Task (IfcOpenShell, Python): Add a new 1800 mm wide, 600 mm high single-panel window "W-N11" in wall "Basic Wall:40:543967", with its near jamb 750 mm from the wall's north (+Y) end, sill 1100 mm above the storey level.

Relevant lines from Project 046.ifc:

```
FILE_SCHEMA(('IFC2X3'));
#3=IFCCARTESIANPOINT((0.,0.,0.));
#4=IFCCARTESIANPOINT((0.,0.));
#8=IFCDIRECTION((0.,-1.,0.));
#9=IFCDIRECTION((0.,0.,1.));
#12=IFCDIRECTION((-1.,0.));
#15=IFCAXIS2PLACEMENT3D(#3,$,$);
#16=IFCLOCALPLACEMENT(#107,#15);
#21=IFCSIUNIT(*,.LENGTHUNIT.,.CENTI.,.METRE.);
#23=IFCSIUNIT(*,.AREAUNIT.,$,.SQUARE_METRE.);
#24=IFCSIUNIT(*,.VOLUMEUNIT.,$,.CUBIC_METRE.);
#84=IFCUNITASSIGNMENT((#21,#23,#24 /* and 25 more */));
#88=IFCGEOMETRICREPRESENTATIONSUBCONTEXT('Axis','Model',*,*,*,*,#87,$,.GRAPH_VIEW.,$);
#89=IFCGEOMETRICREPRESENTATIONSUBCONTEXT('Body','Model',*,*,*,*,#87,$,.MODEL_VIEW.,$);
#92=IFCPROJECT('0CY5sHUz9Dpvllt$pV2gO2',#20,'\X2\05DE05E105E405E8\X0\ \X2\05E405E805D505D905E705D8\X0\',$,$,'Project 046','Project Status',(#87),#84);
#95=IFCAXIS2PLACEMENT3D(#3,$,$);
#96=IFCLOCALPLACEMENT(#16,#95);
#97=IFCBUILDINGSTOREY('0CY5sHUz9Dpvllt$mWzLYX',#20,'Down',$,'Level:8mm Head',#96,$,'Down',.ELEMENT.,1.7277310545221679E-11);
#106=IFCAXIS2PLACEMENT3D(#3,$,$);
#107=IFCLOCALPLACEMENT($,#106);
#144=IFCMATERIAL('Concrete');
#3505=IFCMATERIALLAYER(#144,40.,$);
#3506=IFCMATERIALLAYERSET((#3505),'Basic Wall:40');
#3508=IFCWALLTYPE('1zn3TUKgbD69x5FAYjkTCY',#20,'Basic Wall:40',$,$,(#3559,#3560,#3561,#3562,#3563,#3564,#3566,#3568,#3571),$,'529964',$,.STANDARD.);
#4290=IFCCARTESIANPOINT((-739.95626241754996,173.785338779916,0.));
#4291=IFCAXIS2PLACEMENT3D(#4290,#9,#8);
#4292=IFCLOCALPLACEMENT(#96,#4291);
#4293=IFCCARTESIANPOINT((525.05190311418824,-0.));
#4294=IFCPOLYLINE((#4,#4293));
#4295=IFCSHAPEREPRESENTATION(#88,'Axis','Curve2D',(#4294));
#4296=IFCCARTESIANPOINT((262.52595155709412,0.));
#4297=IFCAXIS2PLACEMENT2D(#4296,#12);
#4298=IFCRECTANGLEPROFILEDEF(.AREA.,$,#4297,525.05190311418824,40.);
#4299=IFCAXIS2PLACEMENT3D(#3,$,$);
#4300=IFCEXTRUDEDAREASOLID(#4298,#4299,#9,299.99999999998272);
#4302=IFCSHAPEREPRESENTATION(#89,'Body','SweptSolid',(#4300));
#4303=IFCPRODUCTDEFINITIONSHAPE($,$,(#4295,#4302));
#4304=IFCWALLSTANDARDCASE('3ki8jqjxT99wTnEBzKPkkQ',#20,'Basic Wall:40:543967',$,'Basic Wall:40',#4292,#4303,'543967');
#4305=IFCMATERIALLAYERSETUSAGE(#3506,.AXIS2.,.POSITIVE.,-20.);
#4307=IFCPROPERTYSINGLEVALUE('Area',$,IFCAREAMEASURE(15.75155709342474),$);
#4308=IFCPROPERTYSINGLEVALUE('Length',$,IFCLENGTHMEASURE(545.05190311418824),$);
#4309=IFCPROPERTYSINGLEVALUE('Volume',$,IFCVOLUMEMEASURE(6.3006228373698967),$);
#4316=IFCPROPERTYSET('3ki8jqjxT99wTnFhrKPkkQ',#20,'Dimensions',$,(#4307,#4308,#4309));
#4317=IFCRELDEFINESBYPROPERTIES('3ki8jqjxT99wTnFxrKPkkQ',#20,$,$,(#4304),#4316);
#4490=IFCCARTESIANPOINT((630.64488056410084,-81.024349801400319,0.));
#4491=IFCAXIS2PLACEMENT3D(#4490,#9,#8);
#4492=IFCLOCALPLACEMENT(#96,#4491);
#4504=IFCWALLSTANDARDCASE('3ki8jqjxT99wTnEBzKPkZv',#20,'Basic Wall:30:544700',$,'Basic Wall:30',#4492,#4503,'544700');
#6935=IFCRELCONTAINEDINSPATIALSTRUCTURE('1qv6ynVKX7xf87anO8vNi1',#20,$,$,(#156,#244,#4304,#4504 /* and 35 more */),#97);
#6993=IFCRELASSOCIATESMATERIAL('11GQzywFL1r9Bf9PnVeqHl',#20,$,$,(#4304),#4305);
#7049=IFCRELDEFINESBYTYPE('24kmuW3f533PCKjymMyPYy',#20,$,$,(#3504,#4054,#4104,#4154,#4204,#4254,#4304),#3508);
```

```python
import numpy as np
import ifcopenshell
import ifcopenshell.api.feature
import ifcopenshell.api.geometry
import ifcopenshell.api.pset
import ifcopenshell.api.root
import ifcopenshell.api.spatial
import ifcopenshell.api.type
import ifcopenshell.geom
import ifcopenshell.util.element
import ifcopenshell.util.placement
import ifcopenshell.util.representation
import ifcopenshell.util.shape
import ifcopenshell.util.unit

model = ifcopenshell.open("Project 046.ifc")
unit_scale = ifcopenshell.util.unit.calculate_unit_scale(model)
area_scale = ifcopenshell.util.unit.calculate_unit_scale(model, "AREAUNIT")
volume_scale = ifcopenshell.util.unit.calculate_unit_scale(model, "VOLUMEUNIT")
settings = ifcopenshell.geom.settings()


def volume(element):
    """Net volume in cubic metres, openings subtracted."""
    shape = ifcopenshell.geom.create_shape(settings, element)
    return ifcopenshell.util.shape.get_volume(shape.geometry)


wall = model.by_guid("3ki8jqjxT99wTnEBzKPkkQ")
storey = ifcopenshell.util.element.get_container(wall, ifc_class="IfcBuildingStorey")
context = ifcopenshell.util.representation.get_context(model, "Model", "Body", "MODEL_VIEW")
before = volume(wall)

width, height, from_end, sill = 1.8, 0.6, 0.75, 1.1  # metres

# The wall runs along its own X axis, and the end named is its -X end.
wall_shape = ifcopenshell.geom.create_shape(settings, wall)
x, y, z = ifcopenshell.util.shape.get_vertices(wall_shape.geometry).T
start = x.min() + from_end
face, thickness = float(y.min()), float(y.max() - y.min())
wall_matrix = ifcopenshell.util.placement.get_local_placement(wall.ObjectPlacement)
level = ifcopenshell.util.placement.get_local_placement(storey.ObjectPlacement)[2, 3]


def in_wall(x, y):
    """Placement at x, y metres in the wall's axes, at sill height."""
    matrix = wall_matrix.copy()
    matrix[:, 3] = wall_matrix @ np.array([x / unit_scale, y / unit_scale, 0.0, 1.0])
    matrix[2, 3] = level + sill / unit_scale
    return matrix


# Opening: a box that overshoots both wall faces by 50 mm.
opening = ifcopenshell.api.root.create_entity(model, ifc_class="IfcOpeningElement")
box = ifcopenshell.api.geometry.add_wall_representation(
    model, context=context, length=width, height=height, thickness=thickness + 0.1
)
ifcopenshell.api.geometry.assign_representation(model, product=opening, representation=box)
ifcopenshell.api.geometry.edit_object_placement(model, product=opening, matrix=in_wall(start, face - 0.05), is_si=False)
ifcopenshell.api.feature.add_feature(model, feature=opening, element=wall)

window = ifcopenshell.api.root.create_entity(model, ifc_class="IfcWindow", name="W-N11")
window.OverallWidth, window.OverallHeight = width / unit_scale, height / unit_scale
body = ifcopenshell.api.geometry.add_window_representation(
    model,
    context=context,
    overall_width=window.OverallWidth,
    overall_height=window.OverallHeight,
    partition_type="SINGLE_PANEL",
)
ifcopenshell.api.geometry.assign_representation(model, product=window, representation=body)
ifcopenshell.api.spatial.assign_container(model, products=[window], relating_structure=storey)
fills = ifcopenshell.api.feature.add_filling(model, opening=opening, element=window)
fills.OwnerHistory = window.OwnerHistory  # required in IFC2X3

# IFC2X3 keeps the operation on the window style.
style = ifcopenshell.api.root.create_entity(model, ifc_class="IfcWindowStyle", name="W-N11")
style.OperationType, style.ConstructionType = "SINGLE_PANEL", "NOTDEFINED"
style.ParameterTakesPrecedence = style.Sizeable = False
ifcopenshell.api.type.assign_type(model, related_objects=[window], relating_type=style)

# Centre the window in the wall's thickness.
ifcopenshell.api.geometry.edit_object_placement(model, product=window, matrix=in_wall(start, face), is_si=False)
window_shape = ifcopenshell.geom.create_shape(settings, window)
depth = ifcopenshell.util.shape.get_vertices(window_shape.geometry)[:, 1]
offset = face + thickness / 2 - (depth.min() + depth.max()) / 2
ifcopenshell.api.geometry.edit_object_placement(model, product=window, matrix=in_wall(start, offset), is_si=False)

after = volume(wall)

# Update the wall's stored quantities.
pset = model.by_id(ifcopenshell.util.element.get_pset(wall, "Dimensions", should_inherit=False)["id"])
ifcopenshell.api.pset.edit_pset(model, pset=pset, properties={
    "Area": model.create_entity("IfcAreaMeasure", after / thickness / area_scale),
    "Volume": model.create_entity("IfcVolumeMeasure", after / volume_scale),
})

print(f"wall volume {before:.3f} -> {after:.3f} m3")

model.write("Project 046_updated.ifc")
```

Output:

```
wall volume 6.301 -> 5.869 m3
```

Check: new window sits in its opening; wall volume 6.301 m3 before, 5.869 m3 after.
